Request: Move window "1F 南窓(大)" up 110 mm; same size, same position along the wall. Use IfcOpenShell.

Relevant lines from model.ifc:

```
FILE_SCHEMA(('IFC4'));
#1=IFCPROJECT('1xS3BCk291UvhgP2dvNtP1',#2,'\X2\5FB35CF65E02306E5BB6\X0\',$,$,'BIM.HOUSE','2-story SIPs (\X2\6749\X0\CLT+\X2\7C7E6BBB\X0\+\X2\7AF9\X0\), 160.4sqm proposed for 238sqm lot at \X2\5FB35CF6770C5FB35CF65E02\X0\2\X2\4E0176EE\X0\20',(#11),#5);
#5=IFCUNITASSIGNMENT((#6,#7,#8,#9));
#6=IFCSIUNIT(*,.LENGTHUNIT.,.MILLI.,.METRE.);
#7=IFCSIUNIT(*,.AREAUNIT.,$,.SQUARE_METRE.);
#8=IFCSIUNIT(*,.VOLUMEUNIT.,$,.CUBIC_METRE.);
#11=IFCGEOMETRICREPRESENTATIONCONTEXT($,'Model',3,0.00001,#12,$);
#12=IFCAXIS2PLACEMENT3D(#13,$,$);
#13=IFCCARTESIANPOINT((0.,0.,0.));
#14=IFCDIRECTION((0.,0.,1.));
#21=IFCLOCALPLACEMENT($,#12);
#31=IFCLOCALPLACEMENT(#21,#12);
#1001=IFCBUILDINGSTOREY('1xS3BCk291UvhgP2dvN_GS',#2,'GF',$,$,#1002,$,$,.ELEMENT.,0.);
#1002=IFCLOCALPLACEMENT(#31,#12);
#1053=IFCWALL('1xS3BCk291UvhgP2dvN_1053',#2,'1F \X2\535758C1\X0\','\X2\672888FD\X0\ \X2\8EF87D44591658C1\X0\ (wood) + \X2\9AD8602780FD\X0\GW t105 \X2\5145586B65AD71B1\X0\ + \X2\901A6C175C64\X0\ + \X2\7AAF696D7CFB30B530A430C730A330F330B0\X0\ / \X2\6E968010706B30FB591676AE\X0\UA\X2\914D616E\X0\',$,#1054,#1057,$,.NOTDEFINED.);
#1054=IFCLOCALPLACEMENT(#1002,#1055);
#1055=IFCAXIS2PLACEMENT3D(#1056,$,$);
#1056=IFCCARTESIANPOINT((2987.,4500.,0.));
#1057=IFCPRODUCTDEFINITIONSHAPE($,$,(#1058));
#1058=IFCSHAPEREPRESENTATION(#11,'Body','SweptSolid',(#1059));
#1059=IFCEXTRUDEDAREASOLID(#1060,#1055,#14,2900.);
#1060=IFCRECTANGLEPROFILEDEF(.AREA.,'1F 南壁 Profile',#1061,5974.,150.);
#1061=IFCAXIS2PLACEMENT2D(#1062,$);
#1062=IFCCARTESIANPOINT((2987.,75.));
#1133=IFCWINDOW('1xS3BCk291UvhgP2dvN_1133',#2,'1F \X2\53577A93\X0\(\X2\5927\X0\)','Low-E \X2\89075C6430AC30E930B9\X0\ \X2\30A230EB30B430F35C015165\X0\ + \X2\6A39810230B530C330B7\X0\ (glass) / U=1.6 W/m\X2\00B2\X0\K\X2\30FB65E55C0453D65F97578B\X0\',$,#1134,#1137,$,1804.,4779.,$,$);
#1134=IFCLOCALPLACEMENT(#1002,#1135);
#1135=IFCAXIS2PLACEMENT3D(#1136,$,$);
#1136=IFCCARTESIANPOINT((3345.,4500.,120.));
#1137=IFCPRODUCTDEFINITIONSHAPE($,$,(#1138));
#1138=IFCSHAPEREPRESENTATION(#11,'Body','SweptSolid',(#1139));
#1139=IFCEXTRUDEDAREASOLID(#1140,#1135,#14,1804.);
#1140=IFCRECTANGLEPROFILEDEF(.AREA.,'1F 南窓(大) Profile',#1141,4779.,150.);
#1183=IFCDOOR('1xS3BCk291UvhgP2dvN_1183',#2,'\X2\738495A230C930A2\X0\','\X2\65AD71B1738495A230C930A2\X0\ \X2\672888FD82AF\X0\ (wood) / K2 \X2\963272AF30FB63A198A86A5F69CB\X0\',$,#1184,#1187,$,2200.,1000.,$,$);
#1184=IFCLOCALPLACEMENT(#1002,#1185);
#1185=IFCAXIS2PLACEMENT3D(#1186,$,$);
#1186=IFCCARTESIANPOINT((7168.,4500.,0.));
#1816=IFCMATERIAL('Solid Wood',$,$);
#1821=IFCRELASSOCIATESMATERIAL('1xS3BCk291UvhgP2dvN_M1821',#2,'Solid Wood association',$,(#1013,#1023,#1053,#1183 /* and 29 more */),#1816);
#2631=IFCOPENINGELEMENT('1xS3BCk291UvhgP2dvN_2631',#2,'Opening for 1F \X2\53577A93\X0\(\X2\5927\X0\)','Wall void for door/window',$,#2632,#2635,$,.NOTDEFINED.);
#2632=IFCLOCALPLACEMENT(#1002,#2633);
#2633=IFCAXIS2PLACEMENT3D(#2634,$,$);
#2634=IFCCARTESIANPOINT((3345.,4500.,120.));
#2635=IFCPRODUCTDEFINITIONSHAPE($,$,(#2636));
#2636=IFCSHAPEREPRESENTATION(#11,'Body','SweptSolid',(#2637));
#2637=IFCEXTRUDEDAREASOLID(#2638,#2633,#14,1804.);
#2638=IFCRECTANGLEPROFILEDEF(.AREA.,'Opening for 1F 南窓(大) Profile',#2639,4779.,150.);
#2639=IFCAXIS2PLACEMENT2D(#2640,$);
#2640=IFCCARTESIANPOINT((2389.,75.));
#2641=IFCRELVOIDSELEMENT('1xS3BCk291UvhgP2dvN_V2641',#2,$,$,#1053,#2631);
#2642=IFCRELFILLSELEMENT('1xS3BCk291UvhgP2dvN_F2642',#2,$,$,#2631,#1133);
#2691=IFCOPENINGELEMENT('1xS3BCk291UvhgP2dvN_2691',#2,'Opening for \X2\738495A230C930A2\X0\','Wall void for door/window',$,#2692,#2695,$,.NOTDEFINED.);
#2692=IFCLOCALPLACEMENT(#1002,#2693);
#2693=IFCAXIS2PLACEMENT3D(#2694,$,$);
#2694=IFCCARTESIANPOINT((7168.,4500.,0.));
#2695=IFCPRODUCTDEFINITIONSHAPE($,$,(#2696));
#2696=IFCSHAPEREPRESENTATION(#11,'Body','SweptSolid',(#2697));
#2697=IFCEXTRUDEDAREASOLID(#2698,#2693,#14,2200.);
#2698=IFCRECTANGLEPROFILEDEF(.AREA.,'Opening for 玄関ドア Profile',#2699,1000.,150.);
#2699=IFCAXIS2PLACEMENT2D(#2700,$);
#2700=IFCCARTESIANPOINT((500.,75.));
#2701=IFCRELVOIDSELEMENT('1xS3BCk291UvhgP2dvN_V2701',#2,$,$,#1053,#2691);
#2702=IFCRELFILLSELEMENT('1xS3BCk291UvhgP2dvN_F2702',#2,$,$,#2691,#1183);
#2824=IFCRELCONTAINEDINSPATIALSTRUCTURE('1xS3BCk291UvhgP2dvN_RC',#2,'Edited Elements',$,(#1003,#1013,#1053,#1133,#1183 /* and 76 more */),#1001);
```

```python
import numpy as np
import ifcopenshell
import ifcopenshell.api.geometry
import ifcopenshell.util.placement
import ifcopenshell.util.unit

model = ifcopenshell.open("model.ifc")
unit_scale = ifcopenshell.util.unit.calculate_unit_scale(model)

window = model.by_guid("1xS3BCk291UvhgP2dvN_1133")
opening = window.FillsVoids[0].RelatingOpeningElement
dz = 0.11 / unit_scale

shift = np.array([0.0, 0.0, dz])
# The window is not placed relative to its opening, so move both.
for product in (opening, window):
    matrix = ifcopenshell.util.placement.get_local_placement(product.ObjectPlacement)
    matrix[:3, 3] += shift
    ifcopenshell.api.geometry.edit_object_placement(model, product=product, matrix=matrix, is_si=False)

print(f"moved by {dz * unit_scale:+.3f} m")

model.write("model_rev.ifc")
```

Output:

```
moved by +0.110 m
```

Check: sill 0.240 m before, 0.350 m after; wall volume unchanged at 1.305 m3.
